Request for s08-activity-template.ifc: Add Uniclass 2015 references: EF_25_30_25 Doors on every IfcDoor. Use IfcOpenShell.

First a look at what the model holds.

```python
import ifcopenshell

model = ifcopenshell.open("s08-activity-template.ifc")
print(model.schema)
print("classifications:", [c.Name for c in model.by_type("IfcClassification")])
for ifc_class in ("IfcDoor", "IfcRoof", "IfcStair", "IfcWall", "IfcWindow"):
    print(ifc_class, len(model.by_type(ifc_class)))
```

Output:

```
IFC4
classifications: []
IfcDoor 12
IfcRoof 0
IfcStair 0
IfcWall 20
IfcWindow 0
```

```python
import ifcopenshell
import ifcopenshell.api.classification

model = ifcopenshell.open("s08-activity-template.ifc")

system = ifcopenshell.api.classification.add_classification(model, classification="Uniclass 2015")

codes = {
    "IfcDoor": ("EF_25_30_25", "Doors"),
}
for ifc_class, (code, name) in codes.items():
    products = model.by_type(ifc_class)
    ifcopenshell.api.classification.add_reference(
        model, products=products, classification=system, identification=code, name=name
    )
    print(code, len(products))

model.write("s08-activity-template_updated.ifc")
```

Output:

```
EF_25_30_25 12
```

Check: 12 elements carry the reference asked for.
